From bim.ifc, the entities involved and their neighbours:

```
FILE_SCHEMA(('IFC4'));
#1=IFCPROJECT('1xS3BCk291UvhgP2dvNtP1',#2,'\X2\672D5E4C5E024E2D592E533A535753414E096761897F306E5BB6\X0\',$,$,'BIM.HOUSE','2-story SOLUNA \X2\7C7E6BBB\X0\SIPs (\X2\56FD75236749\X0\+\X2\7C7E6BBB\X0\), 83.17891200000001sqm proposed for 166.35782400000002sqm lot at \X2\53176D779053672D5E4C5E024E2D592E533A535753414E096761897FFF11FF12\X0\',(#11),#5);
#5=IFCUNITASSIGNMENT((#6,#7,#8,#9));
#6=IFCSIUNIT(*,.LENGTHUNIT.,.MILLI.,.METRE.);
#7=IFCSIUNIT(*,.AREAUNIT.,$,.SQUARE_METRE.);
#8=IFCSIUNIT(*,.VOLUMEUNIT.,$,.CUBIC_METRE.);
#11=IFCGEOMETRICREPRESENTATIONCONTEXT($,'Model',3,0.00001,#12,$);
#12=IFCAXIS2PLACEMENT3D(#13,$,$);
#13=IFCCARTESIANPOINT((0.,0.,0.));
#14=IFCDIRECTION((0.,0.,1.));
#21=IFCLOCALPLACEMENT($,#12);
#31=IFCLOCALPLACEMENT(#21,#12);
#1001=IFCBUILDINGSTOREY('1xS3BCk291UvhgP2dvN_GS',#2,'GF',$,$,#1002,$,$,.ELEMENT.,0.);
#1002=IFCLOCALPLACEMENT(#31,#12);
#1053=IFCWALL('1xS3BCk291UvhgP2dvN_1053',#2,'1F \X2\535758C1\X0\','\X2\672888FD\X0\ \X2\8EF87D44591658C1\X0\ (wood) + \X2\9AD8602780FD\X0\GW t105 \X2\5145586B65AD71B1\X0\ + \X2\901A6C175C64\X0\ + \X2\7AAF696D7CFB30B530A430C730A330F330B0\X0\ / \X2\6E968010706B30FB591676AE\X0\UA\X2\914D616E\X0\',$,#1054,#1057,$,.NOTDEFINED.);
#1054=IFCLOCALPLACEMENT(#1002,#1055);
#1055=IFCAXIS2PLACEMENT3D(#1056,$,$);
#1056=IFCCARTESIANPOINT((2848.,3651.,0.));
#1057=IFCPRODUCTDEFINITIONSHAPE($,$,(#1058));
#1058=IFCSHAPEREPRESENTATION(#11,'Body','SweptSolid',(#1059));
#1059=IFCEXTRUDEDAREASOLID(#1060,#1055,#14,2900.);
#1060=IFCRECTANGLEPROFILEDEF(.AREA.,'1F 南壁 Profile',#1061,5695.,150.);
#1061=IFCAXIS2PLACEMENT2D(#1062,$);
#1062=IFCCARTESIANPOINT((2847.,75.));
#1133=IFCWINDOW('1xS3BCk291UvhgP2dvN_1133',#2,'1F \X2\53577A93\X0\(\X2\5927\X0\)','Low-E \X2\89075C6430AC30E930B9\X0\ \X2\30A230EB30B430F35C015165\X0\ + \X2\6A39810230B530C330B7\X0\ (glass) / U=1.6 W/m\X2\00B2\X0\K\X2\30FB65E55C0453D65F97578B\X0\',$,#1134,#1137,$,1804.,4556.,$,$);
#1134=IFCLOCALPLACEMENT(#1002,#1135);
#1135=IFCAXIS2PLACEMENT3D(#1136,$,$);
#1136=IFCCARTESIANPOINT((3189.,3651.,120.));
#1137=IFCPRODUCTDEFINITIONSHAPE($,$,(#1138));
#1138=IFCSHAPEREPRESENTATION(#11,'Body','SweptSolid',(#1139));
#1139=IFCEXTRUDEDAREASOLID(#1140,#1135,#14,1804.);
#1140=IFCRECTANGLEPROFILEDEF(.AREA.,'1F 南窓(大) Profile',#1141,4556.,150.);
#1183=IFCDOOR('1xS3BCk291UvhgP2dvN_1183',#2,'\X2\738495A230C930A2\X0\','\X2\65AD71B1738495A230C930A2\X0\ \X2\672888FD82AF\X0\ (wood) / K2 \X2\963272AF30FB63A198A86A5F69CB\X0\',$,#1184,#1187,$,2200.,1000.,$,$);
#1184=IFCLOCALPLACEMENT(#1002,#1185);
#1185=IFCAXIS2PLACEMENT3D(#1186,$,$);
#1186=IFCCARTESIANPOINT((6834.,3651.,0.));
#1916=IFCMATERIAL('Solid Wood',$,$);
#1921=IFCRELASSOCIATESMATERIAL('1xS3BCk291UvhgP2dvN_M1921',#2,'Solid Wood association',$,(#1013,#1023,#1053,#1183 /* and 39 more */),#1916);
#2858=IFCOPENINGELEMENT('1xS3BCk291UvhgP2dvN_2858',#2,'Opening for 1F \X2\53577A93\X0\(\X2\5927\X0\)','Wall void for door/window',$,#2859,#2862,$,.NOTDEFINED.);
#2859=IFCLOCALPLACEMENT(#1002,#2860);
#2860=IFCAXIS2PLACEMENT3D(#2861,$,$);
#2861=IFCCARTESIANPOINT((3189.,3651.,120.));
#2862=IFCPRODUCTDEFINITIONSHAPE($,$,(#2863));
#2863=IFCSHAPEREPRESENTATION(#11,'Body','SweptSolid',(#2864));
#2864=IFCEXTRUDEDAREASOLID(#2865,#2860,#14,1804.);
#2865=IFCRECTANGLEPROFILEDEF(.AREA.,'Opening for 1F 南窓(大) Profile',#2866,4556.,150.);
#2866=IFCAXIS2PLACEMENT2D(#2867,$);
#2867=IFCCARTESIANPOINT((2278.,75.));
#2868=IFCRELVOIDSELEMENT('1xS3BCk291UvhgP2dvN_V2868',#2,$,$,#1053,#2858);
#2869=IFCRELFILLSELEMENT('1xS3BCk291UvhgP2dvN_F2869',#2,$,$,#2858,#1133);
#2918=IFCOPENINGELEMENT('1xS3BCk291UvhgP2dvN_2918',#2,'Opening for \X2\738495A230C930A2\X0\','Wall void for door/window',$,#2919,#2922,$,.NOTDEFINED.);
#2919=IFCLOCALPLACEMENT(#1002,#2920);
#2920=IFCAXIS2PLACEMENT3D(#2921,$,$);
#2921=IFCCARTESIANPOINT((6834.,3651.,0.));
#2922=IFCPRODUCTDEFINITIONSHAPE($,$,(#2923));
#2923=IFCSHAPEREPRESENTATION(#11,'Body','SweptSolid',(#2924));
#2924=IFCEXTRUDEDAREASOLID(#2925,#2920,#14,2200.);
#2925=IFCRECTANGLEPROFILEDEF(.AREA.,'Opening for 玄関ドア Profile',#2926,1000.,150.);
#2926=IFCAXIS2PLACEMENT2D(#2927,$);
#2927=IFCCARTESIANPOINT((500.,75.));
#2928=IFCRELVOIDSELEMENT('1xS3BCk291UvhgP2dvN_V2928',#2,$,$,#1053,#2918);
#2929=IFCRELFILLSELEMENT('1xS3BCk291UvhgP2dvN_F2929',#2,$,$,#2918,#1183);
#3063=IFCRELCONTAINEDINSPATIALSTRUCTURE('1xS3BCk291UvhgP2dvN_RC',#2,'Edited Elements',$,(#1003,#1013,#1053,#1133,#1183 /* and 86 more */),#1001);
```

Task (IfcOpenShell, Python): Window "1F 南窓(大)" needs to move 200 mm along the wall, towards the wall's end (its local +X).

```python
import ifcopenshell
import ifcopenshell.api.geometry
import ifcopenshell.util.placement
import ifcopenshell.util.unit

model = ifcopenshell.open("bim.ifc")
unit_scale = ifcopenshell.util.unit.calculate_unit_scale(model)

window = model.by_id(1133)
opening = window.FillsVoids[0].RelatingOpeningElement
wall = opening.VoidsElements[0].RelatingBuildingElement

wall_matrix = ifcopenshell.util.placement.get_local_placement(wall.ObjectPlacement)
shift = wall_matrix[:3, 0] * 0.2 / unit_scale
before = ifcopenshell.util.placement.get_local_placement(window.ObjectPlacement)[:3, 3].copy()

# The window is not placed relative to its opening, so move both.
for product in (opening, window):
    matrix = ifcopenshell.util.placement.get_local_placement(product.ObjectPlacement)
    matrix[:3, 3] += shift
    ifcopenshell.api.geometry.edit_object_placement(model, product=product, matrix=matrix, is_si=False)

after = ifcopenshell.util.placement.get_local_placement(window.ObjectPlacement)[:3, 3]
print("window moved by", (after - before).round(3) + 0.0)

model.write("bim_rev.ifc")
```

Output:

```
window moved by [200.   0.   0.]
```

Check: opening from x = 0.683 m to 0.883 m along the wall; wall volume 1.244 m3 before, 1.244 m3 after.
